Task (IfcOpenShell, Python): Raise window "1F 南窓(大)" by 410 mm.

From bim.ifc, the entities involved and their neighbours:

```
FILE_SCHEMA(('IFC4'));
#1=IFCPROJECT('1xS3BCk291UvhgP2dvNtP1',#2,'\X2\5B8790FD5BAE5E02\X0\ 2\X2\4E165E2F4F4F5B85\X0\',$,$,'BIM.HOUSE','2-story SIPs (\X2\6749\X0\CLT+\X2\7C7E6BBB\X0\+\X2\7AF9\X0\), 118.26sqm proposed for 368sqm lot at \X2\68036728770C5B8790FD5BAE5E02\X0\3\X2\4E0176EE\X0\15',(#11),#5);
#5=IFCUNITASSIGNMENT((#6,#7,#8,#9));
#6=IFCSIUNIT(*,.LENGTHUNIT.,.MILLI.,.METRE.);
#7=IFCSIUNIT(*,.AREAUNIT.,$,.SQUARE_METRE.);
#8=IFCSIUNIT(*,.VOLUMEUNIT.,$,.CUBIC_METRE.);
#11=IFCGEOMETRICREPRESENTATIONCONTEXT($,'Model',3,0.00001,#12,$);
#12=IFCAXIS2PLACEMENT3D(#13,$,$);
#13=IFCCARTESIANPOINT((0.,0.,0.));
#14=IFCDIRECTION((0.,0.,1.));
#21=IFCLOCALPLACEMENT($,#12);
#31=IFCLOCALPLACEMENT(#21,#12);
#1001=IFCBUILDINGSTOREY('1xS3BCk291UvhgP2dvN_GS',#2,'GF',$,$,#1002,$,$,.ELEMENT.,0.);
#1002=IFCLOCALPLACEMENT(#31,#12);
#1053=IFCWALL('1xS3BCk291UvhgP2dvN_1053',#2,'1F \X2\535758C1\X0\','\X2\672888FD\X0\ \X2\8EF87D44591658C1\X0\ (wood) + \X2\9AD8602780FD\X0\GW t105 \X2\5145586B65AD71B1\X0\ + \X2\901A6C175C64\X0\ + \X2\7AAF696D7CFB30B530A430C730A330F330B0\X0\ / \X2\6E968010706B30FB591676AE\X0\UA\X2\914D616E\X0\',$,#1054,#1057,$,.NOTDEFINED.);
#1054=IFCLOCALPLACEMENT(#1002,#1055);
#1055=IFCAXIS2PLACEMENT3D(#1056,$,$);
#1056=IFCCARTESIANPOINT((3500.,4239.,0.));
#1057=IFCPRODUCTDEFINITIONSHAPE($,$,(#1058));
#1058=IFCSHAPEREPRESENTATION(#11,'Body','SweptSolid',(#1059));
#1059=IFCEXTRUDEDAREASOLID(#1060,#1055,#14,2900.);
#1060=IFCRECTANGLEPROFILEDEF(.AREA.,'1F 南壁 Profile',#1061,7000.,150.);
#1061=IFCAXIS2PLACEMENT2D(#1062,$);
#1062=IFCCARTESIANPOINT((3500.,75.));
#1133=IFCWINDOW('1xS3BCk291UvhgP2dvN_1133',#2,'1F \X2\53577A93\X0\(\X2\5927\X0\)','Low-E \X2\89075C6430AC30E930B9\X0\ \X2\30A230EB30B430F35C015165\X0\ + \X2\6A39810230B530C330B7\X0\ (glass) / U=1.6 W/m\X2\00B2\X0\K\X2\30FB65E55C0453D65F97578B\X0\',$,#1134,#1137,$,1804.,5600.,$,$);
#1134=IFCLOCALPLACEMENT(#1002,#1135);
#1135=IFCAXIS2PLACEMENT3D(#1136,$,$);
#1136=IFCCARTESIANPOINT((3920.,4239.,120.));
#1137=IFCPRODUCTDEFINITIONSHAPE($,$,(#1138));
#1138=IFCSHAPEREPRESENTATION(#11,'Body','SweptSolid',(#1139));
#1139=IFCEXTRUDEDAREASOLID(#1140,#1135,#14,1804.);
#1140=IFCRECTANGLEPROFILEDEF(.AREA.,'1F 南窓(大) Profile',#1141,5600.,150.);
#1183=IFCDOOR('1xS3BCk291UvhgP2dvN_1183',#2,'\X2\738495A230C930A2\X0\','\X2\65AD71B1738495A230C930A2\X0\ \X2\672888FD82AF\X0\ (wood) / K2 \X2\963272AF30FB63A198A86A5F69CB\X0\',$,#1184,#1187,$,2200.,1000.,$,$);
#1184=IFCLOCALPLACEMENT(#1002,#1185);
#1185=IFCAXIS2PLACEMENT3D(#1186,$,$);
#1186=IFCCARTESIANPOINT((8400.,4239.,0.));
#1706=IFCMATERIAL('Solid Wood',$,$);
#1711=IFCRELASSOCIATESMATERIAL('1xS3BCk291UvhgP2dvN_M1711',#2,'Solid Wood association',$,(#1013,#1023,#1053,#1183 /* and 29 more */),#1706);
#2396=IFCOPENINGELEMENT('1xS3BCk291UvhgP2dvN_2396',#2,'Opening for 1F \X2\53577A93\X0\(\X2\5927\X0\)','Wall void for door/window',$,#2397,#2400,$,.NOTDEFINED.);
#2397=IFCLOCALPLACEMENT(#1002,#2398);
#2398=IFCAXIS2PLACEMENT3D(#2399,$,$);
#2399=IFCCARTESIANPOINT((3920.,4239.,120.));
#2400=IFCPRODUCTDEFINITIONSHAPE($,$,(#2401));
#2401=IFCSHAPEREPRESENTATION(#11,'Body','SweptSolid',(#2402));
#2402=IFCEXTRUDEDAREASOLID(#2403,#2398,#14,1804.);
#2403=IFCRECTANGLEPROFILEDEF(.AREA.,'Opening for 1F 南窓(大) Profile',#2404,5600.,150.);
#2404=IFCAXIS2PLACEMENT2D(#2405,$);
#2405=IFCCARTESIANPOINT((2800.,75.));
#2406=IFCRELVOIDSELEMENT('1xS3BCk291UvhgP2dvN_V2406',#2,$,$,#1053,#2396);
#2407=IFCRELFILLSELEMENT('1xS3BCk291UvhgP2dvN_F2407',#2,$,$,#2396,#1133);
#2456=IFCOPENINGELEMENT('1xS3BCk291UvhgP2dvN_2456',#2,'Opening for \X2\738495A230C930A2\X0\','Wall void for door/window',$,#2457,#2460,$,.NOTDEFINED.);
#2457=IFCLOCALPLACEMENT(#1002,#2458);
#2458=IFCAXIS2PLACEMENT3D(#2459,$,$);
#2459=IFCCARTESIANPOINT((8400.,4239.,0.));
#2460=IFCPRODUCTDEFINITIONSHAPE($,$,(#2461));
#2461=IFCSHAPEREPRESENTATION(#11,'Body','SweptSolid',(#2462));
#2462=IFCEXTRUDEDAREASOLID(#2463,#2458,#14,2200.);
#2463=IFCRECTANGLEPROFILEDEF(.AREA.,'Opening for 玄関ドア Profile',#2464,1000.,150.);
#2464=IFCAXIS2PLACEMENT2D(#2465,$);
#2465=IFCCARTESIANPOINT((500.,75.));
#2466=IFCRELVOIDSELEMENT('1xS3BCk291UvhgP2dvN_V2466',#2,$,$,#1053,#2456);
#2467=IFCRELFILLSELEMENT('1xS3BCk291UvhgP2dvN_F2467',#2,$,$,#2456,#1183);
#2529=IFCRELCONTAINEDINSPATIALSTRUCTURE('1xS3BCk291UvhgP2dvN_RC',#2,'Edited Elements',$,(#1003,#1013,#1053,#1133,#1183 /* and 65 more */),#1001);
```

```python
import numpy as np
import ifcopenshell
import ifcopenshell.api.geometry
import ifcopenshell.util.placement
import ifcopenshell.util.unit

model = ifcopenshell.open("bim.ifc")
unit_scale = ifcopenshell.util.unit.calculate_unit_scale(model)

window = model.by_guid("1xS3BCk291UvhgP2dvN_1133")
opening = window.FillsVoids[0].RelatingOpeningElement
dz = 0.41 / unit_scale

shift = np.array([0.0, 0.0, dz])
# The window is not placed relative to its opening, so move both.
for product in (opening, window):
    matrix = ifcopenshell.util.placement.get_local_placement(product.ObjectPlacement)
    matrix[:3, 3] += shift
    ifcopenshell.api.geometry.edit_object_placement(model, product=product, matrix=matrix, is_si=False)

print(f"moved by {dz * unit_scale:+.3f} m")

model.write("bim_v2.ifc")
```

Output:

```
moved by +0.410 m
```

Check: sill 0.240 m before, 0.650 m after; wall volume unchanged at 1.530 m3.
